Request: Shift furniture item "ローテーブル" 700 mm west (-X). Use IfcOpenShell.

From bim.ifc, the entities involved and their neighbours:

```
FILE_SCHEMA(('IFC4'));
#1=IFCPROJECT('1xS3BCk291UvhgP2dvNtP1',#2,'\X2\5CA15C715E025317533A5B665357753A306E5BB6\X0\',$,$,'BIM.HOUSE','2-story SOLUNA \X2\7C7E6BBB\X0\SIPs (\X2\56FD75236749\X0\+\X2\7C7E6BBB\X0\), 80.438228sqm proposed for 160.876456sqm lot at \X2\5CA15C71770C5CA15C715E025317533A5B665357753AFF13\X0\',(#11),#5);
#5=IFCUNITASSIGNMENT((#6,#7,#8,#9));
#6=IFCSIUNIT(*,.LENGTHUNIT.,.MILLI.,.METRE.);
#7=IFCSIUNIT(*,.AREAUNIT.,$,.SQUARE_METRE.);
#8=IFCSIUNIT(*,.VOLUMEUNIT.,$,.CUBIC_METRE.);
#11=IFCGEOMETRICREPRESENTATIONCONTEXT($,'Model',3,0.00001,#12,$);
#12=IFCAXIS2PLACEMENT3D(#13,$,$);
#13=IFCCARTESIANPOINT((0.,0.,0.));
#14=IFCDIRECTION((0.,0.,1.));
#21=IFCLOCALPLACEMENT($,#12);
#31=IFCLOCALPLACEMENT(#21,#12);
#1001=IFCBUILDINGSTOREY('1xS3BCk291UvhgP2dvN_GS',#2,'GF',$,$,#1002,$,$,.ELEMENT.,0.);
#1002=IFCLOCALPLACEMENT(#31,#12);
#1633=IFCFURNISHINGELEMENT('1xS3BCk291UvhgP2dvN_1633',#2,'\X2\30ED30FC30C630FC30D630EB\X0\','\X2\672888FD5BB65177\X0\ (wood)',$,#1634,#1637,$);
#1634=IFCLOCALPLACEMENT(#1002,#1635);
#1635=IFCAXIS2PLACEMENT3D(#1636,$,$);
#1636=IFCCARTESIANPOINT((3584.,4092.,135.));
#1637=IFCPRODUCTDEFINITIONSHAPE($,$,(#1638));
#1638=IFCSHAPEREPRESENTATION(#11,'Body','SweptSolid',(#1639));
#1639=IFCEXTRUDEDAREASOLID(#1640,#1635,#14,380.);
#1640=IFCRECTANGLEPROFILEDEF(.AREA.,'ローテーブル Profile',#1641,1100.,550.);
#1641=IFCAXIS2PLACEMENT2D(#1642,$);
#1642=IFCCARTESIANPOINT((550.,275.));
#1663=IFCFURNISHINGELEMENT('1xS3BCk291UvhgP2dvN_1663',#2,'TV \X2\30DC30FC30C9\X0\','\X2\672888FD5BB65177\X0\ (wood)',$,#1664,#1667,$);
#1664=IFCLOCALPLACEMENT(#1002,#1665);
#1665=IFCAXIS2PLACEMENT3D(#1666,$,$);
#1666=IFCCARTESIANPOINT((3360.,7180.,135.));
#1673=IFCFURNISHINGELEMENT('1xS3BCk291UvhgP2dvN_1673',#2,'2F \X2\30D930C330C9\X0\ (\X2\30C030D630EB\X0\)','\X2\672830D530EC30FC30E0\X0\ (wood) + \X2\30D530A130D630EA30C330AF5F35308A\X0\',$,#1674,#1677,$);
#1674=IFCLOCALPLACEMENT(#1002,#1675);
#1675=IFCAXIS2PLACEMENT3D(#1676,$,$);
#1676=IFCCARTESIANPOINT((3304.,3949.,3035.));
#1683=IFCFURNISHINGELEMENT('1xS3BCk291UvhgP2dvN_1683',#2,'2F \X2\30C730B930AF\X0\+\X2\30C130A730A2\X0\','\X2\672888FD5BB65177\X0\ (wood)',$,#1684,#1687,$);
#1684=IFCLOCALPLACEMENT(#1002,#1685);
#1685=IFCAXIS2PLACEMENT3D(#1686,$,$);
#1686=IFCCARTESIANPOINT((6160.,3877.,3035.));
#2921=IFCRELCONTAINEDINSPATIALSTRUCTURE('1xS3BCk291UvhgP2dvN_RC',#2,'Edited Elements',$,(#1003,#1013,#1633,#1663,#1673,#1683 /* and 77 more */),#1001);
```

```python
import ifcopenshell
import ifcopenshell.api.geometry
import ifcopenshell.util.placement
import ifcopenshell.util.unit

model = ifcopenshell.open("bim.ifc")
unit_scale = ifcopenshell.util.unit.calculate_unit_scale(model)

item = model.by_id(1633)
matrix = ifcopenshell.util.placement.get_local_placement(item.ObjectPlacement)
matrix[0, 3] -= 0.7 / unit_scale
ifcopenshell.api.geometry.edit_object_placement(model, product=item, matrix=matrix, is_si=False)

print(ifcopenshell.util.placement.get_local_placement(item.ObjectPlacement).round(3) + 0.0)

model.write("bim-out.ifc")
```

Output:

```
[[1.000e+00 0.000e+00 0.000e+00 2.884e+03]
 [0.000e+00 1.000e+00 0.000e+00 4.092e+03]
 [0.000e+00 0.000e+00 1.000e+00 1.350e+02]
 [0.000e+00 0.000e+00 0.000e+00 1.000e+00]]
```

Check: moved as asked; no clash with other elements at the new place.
